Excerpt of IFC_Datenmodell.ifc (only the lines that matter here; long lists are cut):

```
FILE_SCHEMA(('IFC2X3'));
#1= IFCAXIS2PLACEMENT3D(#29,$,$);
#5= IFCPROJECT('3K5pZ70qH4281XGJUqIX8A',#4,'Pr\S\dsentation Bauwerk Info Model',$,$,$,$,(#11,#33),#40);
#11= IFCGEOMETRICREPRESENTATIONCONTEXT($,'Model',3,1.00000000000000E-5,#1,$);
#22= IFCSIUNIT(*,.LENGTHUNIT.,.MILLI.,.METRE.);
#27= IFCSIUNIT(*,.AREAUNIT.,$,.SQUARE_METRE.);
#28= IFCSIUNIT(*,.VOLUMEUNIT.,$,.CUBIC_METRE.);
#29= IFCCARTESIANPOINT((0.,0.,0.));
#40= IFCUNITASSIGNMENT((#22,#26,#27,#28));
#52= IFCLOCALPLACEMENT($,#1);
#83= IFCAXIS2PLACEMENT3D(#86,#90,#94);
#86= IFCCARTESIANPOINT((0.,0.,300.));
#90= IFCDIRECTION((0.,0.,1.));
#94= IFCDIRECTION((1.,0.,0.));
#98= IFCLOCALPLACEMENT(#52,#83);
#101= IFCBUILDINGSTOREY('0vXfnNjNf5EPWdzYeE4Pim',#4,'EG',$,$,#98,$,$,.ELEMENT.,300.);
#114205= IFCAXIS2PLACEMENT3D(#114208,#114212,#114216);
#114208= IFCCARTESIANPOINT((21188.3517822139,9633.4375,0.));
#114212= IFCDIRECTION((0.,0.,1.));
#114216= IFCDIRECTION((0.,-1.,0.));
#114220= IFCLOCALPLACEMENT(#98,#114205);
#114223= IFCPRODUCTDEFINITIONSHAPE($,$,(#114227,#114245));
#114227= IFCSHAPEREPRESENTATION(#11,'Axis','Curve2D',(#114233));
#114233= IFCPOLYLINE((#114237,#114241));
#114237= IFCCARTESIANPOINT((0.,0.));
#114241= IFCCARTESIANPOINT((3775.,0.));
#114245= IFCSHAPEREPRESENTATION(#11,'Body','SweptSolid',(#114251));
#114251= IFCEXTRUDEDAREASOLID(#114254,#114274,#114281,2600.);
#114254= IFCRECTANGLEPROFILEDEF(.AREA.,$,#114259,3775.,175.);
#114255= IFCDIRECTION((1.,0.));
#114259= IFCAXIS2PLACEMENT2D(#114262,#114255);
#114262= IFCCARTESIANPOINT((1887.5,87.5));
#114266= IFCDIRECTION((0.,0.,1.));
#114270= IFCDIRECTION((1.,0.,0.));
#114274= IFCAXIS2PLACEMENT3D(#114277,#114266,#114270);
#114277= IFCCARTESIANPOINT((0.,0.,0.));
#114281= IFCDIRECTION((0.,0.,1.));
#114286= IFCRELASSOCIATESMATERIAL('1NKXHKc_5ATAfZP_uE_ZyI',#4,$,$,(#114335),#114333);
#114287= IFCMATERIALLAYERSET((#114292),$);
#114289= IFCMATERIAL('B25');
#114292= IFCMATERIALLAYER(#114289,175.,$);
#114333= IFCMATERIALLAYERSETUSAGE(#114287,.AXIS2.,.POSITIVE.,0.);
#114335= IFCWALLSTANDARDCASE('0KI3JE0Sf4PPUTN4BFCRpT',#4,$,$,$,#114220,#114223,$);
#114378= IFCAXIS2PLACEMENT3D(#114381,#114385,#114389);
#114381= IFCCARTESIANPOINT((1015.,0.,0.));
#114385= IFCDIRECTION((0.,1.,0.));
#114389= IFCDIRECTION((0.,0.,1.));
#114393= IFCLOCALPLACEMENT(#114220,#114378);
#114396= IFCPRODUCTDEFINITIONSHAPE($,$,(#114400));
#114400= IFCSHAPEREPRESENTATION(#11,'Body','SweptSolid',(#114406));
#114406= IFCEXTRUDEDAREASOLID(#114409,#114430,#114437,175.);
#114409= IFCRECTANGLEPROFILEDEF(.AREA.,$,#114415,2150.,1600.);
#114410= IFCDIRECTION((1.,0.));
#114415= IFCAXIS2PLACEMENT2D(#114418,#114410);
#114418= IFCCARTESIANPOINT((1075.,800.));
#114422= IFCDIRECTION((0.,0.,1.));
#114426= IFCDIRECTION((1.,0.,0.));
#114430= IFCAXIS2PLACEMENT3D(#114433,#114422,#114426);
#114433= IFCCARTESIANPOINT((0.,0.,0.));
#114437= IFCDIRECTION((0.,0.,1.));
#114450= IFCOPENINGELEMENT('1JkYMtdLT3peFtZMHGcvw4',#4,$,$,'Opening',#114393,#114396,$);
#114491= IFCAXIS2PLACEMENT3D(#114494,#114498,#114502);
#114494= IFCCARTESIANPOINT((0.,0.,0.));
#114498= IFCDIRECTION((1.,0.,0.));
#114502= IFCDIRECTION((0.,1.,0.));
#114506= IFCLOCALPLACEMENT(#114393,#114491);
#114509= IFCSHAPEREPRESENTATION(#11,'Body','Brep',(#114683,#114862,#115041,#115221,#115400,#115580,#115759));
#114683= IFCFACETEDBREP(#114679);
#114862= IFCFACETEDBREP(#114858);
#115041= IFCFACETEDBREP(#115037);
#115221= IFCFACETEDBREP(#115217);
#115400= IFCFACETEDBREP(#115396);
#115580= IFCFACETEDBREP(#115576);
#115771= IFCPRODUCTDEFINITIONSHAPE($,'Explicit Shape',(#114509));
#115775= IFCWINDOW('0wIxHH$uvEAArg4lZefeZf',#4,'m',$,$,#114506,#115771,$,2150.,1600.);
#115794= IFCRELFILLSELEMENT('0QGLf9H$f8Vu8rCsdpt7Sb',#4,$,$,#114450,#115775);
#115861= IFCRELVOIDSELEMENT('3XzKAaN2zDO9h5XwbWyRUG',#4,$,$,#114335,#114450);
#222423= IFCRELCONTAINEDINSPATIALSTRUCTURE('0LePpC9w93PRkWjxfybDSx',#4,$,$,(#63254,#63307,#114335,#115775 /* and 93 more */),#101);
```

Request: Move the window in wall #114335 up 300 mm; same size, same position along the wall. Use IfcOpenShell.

```python
import numpy as np
import ifcopenshell
import ifcopenshell.api.geometry
import ifcopenshell.util.placement
import ifcopenshell.util.unit

model = ifcopenshell.open("IFC_Datenmodell.ifc")
unit_scale = ifcopenshell.util.unit.calculate_unit_scale(model)

window = model.by_guid("0wIxHH$uvEAArg4lZefeZf")
opening = window.FillsVoids[0].RelatingOpeningElement
dz = 0.3 / unit_scale

shift = np.array([0.0, 0.0, dz])
# The window is placed relative to its opening, so it follows when the opening moves.
matrix = ifcopenshell.util.placement.get_local_placement(opening.ObjectPlacement)
matrix[:3, 3] += shift
ifcopenshell.api.geometry.edit_object_placement(
    model, product=opening, matrix=matrix, is_si=False, should_transform_children=True
)

print(f"moved by {dz * unit_scale:+.3f} m")

model.write("IFC_Datenmodell_rev.ifc")
```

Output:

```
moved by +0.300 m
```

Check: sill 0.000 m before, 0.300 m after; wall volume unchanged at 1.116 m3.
